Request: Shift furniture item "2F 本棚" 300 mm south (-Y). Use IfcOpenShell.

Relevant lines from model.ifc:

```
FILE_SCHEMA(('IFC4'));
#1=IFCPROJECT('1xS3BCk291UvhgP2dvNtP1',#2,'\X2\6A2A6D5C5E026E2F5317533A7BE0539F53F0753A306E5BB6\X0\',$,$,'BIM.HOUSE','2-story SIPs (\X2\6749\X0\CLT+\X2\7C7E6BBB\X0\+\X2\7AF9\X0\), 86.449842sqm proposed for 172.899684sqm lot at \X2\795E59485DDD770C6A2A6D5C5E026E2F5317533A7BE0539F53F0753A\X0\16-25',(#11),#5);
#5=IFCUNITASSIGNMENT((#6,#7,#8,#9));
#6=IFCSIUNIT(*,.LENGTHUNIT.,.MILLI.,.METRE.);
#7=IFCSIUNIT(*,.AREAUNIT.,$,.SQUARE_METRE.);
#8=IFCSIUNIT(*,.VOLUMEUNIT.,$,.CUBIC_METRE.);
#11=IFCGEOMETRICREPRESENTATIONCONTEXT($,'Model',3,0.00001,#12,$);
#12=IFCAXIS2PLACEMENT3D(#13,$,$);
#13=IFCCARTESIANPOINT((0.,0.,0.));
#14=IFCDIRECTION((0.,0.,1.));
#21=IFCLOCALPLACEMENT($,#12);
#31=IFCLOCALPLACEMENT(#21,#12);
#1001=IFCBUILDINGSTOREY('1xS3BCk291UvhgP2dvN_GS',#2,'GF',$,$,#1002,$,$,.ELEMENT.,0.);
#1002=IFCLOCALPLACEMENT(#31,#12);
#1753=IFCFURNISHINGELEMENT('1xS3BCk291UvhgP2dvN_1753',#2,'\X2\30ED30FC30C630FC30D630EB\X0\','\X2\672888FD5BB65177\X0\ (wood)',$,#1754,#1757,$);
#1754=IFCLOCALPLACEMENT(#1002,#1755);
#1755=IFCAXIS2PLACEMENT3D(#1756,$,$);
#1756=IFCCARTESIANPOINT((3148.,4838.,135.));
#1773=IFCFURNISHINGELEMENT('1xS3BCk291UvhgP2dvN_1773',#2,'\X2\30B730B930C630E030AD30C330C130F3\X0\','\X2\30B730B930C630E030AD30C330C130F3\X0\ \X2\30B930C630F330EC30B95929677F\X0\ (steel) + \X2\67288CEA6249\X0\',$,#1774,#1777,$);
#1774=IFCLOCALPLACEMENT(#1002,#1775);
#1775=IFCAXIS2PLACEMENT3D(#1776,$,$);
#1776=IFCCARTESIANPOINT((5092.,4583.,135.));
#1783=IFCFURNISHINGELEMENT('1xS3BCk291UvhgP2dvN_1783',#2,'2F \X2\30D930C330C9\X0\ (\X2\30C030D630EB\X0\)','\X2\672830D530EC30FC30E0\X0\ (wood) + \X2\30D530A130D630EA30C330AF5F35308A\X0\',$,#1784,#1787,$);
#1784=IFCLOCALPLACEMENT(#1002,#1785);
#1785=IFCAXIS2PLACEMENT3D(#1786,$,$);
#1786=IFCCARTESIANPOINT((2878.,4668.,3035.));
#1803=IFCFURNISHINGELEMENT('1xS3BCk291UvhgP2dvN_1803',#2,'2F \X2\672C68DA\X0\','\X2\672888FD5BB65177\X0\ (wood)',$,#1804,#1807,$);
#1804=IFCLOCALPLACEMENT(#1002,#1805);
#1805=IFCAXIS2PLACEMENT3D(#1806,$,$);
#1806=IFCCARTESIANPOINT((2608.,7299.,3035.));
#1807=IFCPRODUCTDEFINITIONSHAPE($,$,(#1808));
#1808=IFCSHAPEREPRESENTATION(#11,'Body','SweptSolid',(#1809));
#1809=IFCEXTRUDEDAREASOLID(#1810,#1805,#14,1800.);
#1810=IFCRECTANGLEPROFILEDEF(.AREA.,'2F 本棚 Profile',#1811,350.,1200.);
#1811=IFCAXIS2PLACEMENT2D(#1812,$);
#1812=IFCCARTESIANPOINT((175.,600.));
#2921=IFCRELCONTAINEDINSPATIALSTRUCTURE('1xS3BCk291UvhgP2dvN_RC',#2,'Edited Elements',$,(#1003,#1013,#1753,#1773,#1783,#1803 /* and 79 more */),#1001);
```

```python
import ifcopenshell
import ifcopenshell.api.geometry
import ifcopenshell.util.placement

model = ifcopenshell.open("model.ifc")

item = model.by_guid("1xS3BCk291UvhgP2dvN_1803")
matrix = ifcopenshell.util.placement.get_local_placement(item.ObjectPlacement)
matrix[1, 3] -= 300.0
ifcopenshell.api.geometry.edit_object_placement(model, product=item, matrix=matrix, is_si=False)

print(ifcopenshell.util.placement.get_local_placement(item.ObjectPlacement).round(3) + 0.0)

model.write("model_rev.ifc")
```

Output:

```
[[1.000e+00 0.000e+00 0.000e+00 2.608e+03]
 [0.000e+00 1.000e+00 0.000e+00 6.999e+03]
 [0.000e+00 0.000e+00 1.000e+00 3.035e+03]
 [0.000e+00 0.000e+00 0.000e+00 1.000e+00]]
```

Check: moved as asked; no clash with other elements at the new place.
